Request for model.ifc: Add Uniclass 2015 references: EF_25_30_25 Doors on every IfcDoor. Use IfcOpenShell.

First a look at what the model holds.

```python
import ifcopenshell

model = ifcopenshell.open("model.ifc")
print(model.schema)
print("classifications:", [c.Name for c in model.by_type("IfcClassification")])
for ifc_class in ("IfcDoor", "IfcRoof", "IfcStair", "IfcWall", "IfcWindow"):
    print(ifc_class, len(model.by_type(ifc_class)))
```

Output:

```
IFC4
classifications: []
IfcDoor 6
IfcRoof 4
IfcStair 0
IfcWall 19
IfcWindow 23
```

```python
import ifcopenshell
import ifcopenshell.api.classification

model = ifcopenshell.open("model.ifc")

system = ifcopenshell.api.classification.add_classification(model, classification="Uniclass 2015")

codes = {
    "IfcDoor": ("EF_25_30_25", "Doors"),
}
for ifc_class, (code, name) in codes.items():
    products = model.by_type(ifc_class)
    ifcopenshell.api.classification.add_reference(
        model, products=products, classification=system, identification=code, name=name
    )
    print(code, len(products))

model.write("model_updated.ifc")
```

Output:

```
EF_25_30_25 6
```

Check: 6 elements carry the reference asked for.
